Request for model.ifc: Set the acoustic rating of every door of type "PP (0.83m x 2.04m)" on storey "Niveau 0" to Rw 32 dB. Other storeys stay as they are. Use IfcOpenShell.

First a look at what the model holds.

```python
import ifcopenshell
import ifcopenshell.util.element

model = ifcopenshell.open("model.ifc")
print(model.schema)
storey = next(s for s in model.by_type("IfcBuildingStorey") if s.Name == "Niveau 0")
doors = [e for e in ifcopenshell.util.element.get_decomposition(storey) if e.is_a("IfcDoor")]
seen = {}
for e in doors:
    element_type = ifcopenshell.util.element.get_type(e)
    key = (element_type.Name if element_type != e and element_type else None, ifcopenshell.util.element.get_pset(e, "Pset_DoorCommon", "AcousticRating"))
    seen[key] = seen.get(key, 0) + 1
for (name, value), count in sorted(seen.items(), key=str):
    print(count, "x", name, "|", value)
```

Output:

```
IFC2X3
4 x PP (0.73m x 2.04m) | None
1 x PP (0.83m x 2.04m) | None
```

```python
import ifcopenshell
import ifcopenshell.api.pset
import ifcopenshell.util.element

model = ifcopenshell.open("model.ifc")

storey = next(s for s in model.by_type("IfcBuildingStorey") if s.Name == "Niveau 0")
doors = [e for e in ifcopenshell.util.element.get_decomposition(storey) if e.is_a("IfcDoor")]

count = 0
for e in doors:
    element_type = ifcopenshell.util.element.get_type(e)
    if element_type in (None, e) or element_type.Name != "PP (0.83m x 2.04m)":
        continue
    # add_pset returns the element's existing set when there is one.
    pset = ifcopenshell.api.pset.add_pset(model, product=e, name="Pset_DoorCommon")
    ifcopenshell.api.pset.edit_pset(model, pset=pset, properties={"AcousticRating": "Rw 32 dB"})
    count += 1

print(count, "doors updated")

model.write("model_v2.ifc")
```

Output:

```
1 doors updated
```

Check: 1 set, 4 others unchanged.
